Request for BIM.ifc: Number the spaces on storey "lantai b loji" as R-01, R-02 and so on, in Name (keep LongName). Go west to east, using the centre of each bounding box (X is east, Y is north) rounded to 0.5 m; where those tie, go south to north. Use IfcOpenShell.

First a look at what the model holds.

```python
import ifcopenshell
import ifcopenshell.util.element
import ifcopenshell.util.placement

model = ifcopenshell.open("BIM.ifc")
print(model.schema)
storey = next(s for s in model.by_type("IfcBuildingStorey") if s.Name == "lantai b loji")
spaces = [e for e in ifcopenshell.util.element.get_decomposition(storey) if e.is_a("IfcSpace")]
for e in sorted(spaces, key=lambda e: e.id()):
    origin = ifcopenshell.util.placement.get_local_placement(e.ObjectPlacement)[:3, 3]
    print(e.id(), e.Name, e.LongName, origin.round(2) + 0.0, sep=" | ")
```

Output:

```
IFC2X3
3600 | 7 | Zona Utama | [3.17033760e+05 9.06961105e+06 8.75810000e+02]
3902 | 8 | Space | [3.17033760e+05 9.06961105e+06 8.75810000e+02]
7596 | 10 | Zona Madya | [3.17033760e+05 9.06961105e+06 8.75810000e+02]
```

```python
import ifcopenshell
import ifcopenshell.geom
import ifcopenshell.util.element
import ifcopenshell.util.shape

model = ifcopenshell.open("BIM.ifc")
settings = ifcopenshell.geom.settings()
settings.set("use-world-coords", True)


def centre(element):
    shape = ifcopenshell.geom.create_shape(settings, element)
    return ifcopenshell.util.shape.get_bbox_centroid(shape.geometry)


storey = next(s for s in model.by_type("IfcBuildingStorey") if s.Name == "lantai b loji")
spaces = [e for e in ifcopenshell.util.element.get_decomposition(storey) if e.is_a("IfcSpace")]

# Insertion points can sit at a corner or the storey origin, so sort by the geometry (in metres).
centres = {e: centre(e) for e in spaces}
spaces.sort(key=lambda e: (round(centres[e][0] / 0.5), centres[e][1]))

for i, e in enumerate(spaces, start=1):
    number = f"R-{i:02d}"
    e.Name = number
    print(e.id(), number)

model.write("BIM_updated.ifc")
```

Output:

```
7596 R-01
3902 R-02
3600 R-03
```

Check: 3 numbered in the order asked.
